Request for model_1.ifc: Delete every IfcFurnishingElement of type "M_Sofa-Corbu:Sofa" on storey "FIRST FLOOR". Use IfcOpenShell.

First a look at what the model holds.

```python
import ifcopenshell
import ifcopenshell.util.element

model = ifcopenshell.open("model_1.ifc")
print(model.schema)
storey = next(s for s in model.by_type("IfcBuildingStorey") if s.Name == "FIRST FLOOR")
furniture = [e for e in ifcopenshell.util.element.get_decomposition(storey) if e.is_a("IfcFurnishingElement")]
seen = {}
for e in furniture:
    element_type = ifcopenshell.util.element.get_type(e)
    name = element_type.Name if element_type not in (None, e) else None
    seen[name] = seen.get(name, 0) + 1
for name, count in sorted(seen.items(), key=str):
    print(count, "x", name)
```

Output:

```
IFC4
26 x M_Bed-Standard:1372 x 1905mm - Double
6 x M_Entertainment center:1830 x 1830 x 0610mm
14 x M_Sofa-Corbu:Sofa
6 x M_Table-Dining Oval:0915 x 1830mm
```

```python
import ifcopenshell
import ifcopenshell.api.root
import ifcopenshell.util.element

model = ifcopenshell.open("model_1.ifc")

storey = next(s for s in model.by_type("IfcBuildingStorey") if s.Name == "FIRST FLOOR")
furniture = [e for e in ifcopenshell.util.element.get_decomposition(storey) if e.is_a("IfcFurnishingElement")]
targets = [e for e in furniture if (t := ifcopenshell.util.element.get_type(e)) not in (None, e) and t.Name == "M_Sofa-Corbu:Sofa"]

for e in targets:
    ifcopenshell.api.root.remove_product(model, product=e)
print(len(targets), "removed")

model.write("model_1_v2.ifc")
```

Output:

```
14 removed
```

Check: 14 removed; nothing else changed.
